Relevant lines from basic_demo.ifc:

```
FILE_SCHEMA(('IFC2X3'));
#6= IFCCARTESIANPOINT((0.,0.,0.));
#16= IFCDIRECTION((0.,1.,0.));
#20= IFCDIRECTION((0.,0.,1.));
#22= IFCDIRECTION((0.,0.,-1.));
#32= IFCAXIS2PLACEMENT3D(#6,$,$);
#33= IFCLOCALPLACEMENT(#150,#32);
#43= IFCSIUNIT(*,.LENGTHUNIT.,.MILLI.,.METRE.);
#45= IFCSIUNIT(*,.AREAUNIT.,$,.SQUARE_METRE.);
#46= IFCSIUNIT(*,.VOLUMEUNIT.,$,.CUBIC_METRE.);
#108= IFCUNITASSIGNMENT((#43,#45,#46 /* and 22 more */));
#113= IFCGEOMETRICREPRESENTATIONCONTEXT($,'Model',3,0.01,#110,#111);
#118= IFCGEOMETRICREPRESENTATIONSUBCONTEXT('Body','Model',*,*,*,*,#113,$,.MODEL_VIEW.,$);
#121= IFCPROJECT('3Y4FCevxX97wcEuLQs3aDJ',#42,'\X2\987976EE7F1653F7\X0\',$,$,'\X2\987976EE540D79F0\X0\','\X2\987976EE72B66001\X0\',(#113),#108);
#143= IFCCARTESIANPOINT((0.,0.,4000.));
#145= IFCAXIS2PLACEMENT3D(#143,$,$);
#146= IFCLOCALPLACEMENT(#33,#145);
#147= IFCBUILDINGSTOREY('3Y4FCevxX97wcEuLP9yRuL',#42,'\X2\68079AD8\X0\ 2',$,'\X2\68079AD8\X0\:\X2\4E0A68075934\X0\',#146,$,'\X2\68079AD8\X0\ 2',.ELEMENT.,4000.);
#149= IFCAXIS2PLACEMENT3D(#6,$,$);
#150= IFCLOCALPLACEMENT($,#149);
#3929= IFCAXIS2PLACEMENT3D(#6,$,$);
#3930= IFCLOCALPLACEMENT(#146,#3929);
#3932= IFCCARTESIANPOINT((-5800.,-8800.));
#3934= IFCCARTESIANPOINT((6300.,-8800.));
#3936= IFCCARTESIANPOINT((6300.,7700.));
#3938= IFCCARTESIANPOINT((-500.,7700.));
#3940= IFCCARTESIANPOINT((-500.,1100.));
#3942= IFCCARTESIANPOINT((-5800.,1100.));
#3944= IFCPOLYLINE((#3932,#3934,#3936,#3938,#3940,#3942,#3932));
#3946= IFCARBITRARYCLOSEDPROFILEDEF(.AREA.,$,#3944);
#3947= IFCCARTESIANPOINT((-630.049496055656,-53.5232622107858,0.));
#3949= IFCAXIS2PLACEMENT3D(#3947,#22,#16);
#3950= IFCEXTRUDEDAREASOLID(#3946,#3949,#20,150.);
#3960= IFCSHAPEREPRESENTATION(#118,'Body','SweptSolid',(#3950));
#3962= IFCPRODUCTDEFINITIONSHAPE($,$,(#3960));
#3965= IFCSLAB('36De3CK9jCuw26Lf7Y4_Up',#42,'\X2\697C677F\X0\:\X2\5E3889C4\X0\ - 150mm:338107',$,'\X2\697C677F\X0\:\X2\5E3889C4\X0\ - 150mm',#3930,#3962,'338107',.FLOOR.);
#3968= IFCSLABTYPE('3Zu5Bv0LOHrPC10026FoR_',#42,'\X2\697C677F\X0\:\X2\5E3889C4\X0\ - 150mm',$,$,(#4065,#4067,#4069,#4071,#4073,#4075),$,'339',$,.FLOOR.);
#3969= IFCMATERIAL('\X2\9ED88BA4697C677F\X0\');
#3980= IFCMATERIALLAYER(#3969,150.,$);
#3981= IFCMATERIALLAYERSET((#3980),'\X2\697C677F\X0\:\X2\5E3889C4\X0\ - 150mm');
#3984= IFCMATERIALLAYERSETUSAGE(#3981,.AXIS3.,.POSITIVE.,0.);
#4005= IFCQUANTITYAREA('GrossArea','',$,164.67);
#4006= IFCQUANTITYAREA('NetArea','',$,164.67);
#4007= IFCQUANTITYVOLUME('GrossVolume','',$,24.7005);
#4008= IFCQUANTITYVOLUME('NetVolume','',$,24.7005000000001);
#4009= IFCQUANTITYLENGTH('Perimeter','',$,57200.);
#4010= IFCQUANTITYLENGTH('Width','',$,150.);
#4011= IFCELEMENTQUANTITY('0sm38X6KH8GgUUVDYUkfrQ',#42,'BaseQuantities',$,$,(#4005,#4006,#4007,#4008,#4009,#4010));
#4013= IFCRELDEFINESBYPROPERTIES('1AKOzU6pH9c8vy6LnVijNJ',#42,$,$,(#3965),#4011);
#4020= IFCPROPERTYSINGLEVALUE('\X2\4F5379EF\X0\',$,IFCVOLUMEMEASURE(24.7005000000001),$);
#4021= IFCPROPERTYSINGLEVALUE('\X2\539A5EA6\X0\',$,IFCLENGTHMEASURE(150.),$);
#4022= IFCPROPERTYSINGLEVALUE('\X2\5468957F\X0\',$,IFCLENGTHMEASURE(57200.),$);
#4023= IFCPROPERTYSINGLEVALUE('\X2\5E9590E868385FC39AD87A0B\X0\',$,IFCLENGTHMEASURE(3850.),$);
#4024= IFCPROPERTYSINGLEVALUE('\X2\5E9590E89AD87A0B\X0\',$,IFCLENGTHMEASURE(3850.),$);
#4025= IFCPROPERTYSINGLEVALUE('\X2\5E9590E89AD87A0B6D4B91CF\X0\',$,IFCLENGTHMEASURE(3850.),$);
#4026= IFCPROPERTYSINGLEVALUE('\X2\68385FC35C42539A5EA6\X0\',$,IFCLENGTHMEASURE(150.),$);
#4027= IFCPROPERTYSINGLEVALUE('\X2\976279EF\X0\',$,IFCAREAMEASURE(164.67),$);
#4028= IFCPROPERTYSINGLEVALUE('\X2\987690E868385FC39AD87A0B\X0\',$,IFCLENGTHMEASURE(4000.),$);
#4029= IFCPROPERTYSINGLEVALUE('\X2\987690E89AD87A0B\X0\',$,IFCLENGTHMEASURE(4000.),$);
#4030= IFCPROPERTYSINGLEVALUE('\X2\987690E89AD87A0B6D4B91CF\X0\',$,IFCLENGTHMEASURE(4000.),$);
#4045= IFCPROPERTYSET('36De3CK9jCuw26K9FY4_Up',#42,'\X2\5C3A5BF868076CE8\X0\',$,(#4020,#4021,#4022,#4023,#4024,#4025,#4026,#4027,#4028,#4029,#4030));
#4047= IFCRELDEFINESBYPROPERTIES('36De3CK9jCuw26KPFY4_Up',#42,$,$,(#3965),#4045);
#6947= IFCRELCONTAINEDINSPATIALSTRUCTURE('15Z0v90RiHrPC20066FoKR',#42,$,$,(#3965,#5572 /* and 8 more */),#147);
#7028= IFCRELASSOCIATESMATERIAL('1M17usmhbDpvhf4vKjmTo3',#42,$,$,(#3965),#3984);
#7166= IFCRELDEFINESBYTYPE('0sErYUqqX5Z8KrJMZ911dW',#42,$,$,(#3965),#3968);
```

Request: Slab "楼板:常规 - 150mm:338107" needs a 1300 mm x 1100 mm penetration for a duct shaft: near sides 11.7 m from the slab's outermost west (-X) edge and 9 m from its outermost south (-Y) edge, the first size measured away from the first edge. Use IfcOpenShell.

```python
import numpy as np
import ifcopenshell
import ifcopenshell.api.feature
import ifcopenshell.api.geometry
import ifcopenshell.api.pset
import ifcopenshell.api.root
import ifcopenshell.geom
import ifcopenshell.util.element
import ifcopenshell.util.placement
import ifcopenshell.util.representation
import ifcopenshell.util.shape
import ifcopenshell.util.unit

model = ifcopenshell.open("basic_demo.ifc")
unit_scale = ifcopenshell.util.unit.calculate_unit_scale(model)
area_scale = ifcopenshell.util.unit.calculate_unit_scale(model, "AREAUNIT")
volume_scale = ifcopenshell.util.unit.calculate_unit_scale(model, "VOLUMEUNIT")
settings = ifcopenshell.geom.settings()


def volume(element):
    """Net volume in cubic metres, openings subtracted."""
    shape = ifcopenshell.geom.create_shape(settings, element)
    return ifcopenshell.util.shape.get_volume(shape.geometry)


slab = model.by_guid("36De3CK9jCuw26Lf7Y4_Up")
before = volume(slab)

# Extent in the slab's own axes, in metres. The edges named are its -X and -Y sides.
slab_shape = ifcopenshell.geom.create_shape(settings, slab)
vertices = ifcopenshell.util.shape.get_vertices(slab_shape.geometry)
x_min, y_min, bottom = vertices.min(axis=0)
top = vertices[:, 2].max()

opening = ifcopenshell.api.root.create_entity(model, ifc_class="IfcOpeningElement", name="Duct shaft opening")
context = ifcopenshell.util.representation.get_context(model, "Model", "Body", "MODEL_VIEW")
width, depth = 1.3, 1.1
outline = [(0.0, 0.0), (width, 0.0), (width, depth), (0.0, depth), (0.0, 0.0)]
# Overshoot both faces by 50 mm so the cut is clean.
shape = ifcopenshell.api.geometry.add_slab_representation(
    model, context=context, depth=top - bottom + 0.1, polyline=outline
)
ifcopenshell.api.geometry.assign_representation(model, product=opening, representation=shape)

matrix = ifcopenshell.util.placement.get_local_placement(slab.ObjectPlacement)
matrix[:, 3] = matrix @ np.append(np.array([x_min + 11.7, y_min + 9, bottom - 0.05]) / unit_scale, 1.0)
ifcopenshell.api.geometry.edit_object_placement(model, product=opening, matrix=matrix, is_si=False)
ifcopenshell.api.feature.add_feature(model, feature=opening, element=slab)

after = volume(slab)

# Update the slab's stored quantities.
qto = model.by_id(ifcopenshell.util.element.get_pset(slab, "BaseQuantities", should_inherit=False)["id"])
ifcopenshell.api.pset.edit_qto(model, qto=qto, properties={
    "NetArea": after / (top - bottom) / area_scale,
    "NetVolume": after / volume_scale,
})
pset = model.by_id(ifcopenshell.util.element.get_pset(slab, "尺寸标注", should_inherit=False)["id"])
ifcopenshell.api.pset.edit_pset(model, pset=pset, properties={
    "体积": model.create_entity("IfcVolumeMeasure", after / volume_scale),
    "面积": model.create_entity("IfcAreaMeasure", after / (top - bottom) / area_scale),
})

print(f"slab volume {before:.3f} -> {after:.3f} m3")

model.write("basic_demo_updated.ifc")
```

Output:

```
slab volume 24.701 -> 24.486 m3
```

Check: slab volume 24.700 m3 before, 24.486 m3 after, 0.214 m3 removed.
